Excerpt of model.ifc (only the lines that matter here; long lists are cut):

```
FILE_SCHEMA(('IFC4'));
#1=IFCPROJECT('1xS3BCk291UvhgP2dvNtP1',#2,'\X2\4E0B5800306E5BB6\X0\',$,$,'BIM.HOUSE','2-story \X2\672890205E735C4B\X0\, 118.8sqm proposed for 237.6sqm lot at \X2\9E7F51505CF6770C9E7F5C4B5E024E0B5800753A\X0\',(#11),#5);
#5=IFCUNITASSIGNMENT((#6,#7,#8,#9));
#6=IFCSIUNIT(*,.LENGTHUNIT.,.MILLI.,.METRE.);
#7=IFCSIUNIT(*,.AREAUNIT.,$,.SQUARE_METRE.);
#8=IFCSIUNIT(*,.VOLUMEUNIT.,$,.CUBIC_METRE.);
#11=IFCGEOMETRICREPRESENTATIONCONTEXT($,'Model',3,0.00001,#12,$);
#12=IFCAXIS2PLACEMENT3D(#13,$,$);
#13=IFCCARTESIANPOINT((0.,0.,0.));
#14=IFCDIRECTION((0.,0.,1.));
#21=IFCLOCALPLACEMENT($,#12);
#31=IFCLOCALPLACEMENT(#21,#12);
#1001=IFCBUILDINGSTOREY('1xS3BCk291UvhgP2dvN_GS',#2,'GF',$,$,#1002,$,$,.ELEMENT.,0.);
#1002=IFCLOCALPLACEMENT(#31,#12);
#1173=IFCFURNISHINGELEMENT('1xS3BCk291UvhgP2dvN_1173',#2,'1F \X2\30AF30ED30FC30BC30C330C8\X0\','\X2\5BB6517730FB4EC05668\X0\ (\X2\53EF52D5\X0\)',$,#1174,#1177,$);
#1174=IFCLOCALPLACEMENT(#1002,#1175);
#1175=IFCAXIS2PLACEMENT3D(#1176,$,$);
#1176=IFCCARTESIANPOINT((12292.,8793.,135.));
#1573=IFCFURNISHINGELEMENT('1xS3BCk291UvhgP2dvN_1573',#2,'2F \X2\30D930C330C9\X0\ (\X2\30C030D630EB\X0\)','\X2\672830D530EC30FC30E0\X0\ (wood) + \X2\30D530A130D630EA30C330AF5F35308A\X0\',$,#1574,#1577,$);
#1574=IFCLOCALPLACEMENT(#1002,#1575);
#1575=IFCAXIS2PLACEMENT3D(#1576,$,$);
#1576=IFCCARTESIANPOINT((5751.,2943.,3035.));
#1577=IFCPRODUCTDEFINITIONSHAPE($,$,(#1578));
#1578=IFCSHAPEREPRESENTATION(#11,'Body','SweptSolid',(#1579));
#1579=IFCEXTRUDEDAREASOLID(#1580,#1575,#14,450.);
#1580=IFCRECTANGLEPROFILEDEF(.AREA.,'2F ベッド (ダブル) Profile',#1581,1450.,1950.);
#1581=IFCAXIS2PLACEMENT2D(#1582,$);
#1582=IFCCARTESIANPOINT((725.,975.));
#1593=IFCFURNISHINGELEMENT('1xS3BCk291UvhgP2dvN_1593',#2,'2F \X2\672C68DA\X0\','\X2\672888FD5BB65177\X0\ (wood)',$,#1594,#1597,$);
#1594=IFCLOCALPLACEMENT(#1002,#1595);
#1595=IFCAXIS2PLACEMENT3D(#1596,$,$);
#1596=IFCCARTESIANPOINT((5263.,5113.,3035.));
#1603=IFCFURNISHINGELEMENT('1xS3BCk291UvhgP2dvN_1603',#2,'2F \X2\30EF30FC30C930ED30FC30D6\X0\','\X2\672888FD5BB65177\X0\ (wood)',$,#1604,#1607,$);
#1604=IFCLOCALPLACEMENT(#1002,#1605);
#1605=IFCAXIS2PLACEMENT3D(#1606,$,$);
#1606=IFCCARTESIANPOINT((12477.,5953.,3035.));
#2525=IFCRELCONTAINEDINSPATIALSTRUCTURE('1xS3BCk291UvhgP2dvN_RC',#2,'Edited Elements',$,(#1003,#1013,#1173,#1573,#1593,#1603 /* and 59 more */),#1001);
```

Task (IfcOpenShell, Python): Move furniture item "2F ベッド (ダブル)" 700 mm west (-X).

```python
import ifcopenshell
import ifcopenshell.api.geometry
import ifcopenshell.util.placement
import ifcopenshell.util.unit

model = ifcopenshell.open("model.ifc")
unit_scale = ifcopenshell.util.unit.calculate_unit_scale(model)

item = model.by_guid("1xS3BCk291UvhgP2dvN_1573")
matrix = ifcopenshell.util.placement.get_local_placement(item.ObjectPlacement)
matrix[0, 3] -= 0.7 / unit_scale
ifcopenshell.api.geometry.edit_object_placement(model, product=item, matrix=matrix, is_si=False)

print(ifcopenshell.util.placement.get_local_placement(item.ObjectPlacement).round(3) + 0.0)

model.write("model_updated.ifc")
```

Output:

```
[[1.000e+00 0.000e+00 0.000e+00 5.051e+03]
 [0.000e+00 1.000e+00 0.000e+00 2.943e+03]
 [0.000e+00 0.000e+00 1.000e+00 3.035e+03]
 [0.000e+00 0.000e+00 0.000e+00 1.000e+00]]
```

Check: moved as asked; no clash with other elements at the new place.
